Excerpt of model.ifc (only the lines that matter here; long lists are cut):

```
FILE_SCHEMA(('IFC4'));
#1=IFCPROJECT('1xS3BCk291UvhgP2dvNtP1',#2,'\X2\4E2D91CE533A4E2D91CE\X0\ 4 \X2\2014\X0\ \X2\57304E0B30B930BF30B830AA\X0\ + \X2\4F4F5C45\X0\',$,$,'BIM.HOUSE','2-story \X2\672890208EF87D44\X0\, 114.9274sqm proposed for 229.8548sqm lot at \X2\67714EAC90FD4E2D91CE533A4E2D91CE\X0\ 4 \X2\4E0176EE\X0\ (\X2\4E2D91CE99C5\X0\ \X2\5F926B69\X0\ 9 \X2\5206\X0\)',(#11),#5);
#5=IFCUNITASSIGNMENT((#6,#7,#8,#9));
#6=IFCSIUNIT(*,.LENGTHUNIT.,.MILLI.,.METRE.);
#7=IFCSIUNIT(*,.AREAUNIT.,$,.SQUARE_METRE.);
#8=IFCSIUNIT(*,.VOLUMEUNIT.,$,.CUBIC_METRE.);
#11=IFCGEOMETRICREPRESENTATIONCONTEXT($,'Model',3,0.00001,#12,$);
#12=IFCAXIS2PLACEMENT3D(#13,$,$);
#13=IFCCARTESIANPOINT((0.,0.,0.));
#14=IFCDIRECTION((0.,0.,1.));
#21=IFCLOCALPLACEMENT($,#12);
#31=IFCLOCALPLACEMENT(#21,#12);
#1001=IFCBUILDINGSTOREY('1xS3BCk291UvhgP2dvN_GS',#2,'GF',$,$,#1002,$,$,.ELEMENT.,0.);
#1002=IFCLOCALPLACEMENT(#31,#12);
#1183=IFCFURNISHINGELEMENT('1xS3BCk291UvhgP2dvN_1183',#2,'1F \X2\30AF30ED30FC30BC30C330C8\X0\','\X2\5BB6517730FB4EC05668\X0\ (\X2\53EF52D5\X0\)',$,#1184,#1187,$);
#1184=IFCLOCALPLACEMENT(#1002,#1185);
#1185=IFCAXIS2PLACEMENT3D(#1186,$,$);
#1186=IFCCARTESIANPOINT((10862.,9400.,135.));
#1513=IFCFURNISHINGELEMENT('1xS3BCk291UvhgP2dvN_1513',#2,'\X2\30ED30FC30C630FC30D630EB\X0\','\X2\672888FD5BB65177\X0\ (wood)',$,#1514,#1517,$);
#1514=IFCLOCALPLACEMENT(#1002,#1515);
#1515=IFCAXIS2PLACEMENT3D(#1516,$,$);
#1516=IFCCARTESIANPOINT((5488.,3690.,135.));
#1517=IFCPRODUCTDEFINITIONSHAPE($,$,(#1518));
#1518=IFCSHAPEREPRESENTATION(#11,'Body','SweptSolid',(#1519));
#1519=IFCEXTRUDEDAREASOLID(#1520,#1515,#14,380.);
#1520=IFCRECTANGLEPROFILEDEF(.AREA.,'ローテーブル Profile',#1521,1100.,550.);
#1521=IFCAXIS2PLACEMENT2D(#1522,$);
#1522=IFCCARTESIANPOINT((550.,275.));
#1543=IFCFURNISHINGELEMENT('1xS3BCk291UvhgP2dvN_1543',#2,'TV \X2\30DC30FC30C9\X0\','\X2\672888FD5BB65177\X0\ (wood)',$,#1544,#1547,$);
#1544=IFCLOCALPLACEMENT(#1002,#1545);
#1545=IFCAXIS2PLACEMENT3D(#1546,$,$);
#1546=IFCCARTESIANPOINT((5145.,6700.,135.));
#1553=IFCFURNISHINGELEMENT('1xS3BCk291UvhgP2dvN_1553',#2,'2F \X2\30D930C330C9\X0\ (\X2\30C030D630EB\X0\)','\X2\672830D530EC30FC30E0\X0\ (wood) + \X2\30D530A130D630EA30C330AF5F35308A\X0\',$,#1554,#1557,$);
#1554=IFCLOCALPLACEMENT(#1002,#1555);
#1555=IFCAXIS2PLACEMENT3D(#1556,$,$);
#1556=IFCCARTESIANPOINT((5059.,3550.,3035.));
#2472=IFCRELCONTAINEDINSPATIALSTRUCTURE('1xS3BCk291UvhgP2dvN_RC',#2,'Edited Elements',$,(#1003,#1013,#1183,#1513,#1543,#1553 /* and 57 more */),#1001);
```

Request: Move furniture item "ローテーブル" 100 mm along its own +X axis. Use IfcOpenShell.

```python
import ifcopenshell
import ifcopenshell.api.geometry
import ifcopenshell.util.placement
import ifcopenshell.util.unit

model = ifcopenshell.open("model.ifc")
unit_scale = ifcopenshell.util.unit.calculate_unit_scale(model)

item = model.by_id(1513)
matrix = ifcopenshell.util.placement.get_local_placement(item.ObjectPlacement)
matrix[:3, 3] += matrix[:3, 0] * 0.1 / unit_scale
ifcopenshell.api.geometry.edit_object_placement(model, product=item, matrix=matrix, is_si=False)

print(ifcopenshell.util.placement.get_local_placement(item.ObjectPlacement).round(3) + 0.0)

model.write("model_updated.ifc")
```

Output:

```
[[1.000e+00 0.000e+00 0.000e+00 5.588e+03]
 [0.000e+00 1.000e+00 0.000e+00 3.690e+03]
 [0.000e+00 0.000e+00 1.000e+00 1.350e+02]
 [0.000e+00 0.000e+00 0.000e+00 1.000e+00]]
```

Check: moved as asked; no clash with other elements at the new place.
